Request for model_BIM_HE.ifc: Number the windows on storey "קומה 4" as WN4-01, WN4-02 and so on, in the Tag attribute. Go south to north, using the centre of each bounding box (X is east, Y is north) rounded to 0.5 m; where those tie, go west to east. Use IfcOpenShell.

First a look at what the model holds.

```python
import ifcopenshell
import ifcopenshell.util.element
import ifcopenshell.util.placement

model = ifcopenshell.open("model_BIM_HE.ifc")
print(model.schema)
storey = next(s for s in model.by_type("IfcBuildingStorey") if s.Name == "קומה 4")
windows = [e for e in ifcopenshell.util.element.get_decomposition(storey) if e.is_a("IfcWindow")]
for e in sorted(windows, key=lambda e: e.id()):
    origin = ifcopenshell.util.placement.get_local_placement(e.ObjectPlacement)[:3, 3]
    print(e.id(), e.Tag, e.Name, origin.round(2) + 0.0, sep=" | ")
```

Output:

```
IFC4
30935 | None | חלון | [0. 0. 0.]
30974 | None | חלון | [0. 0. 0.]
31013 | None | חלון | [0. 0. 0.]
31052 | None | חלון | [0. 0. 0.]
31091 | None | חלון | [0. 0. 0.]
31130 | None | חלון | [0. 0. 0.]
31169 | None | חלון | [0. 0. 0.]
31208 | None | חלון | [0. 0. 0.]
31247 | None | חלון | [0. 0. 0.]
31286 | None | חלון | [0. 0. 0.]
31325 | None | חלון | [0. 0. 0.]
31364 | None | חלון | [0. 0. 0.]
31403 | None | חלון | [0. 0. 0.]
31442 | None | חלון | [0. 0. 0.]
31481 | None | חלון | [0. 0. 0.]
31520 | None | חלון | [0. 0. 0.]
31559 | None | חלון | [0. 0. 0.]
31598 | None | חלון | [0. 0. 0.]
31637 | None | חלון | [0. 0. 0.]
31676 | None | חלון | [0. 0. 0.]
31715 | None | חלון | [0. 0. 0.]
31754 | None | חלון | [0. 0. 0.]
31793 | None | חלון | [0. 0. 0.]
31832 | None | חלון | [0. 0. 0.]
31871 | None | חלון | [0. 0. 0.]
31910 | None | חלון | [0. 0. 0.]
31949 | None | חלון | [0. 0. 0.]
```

```python
import ifcopenshell
import ifcopenshell.geom
import ifcopenshell.util.element
import ifcopenshell.util.shape

model = ifcopenshell.open("model_BIM_HE.ifc")
settings = ifcopenshell.geom.settings()
settings.set("use-world-coords", True)


def centre(element):
    shape = ifcopenshell.geom.create_shape(settings, element)
    return ifcopenshell.util.shape.get_bbox_centroid(shape.geometry)


storey = next(s for s in model.by_type("IfcBuildingStorey") if s.Name == "קומה 4")
windows = [e for e in ifcopenshell.util.element.get_decomposition(storey) if e.is_a("IfcWindow")]

# Insertion points can sit at a corner or the storey origin, so sort by the geometry (in metres).
centres = {e: centre(e) for e in windows}
windows.sort(key=lambda e: (round(centres[e][1] / 0.5), centres[e][0]))

for i, e in enumerate(windows, start=1):
    number = f"WN4-{i:02d}"
    e.Tag = number
    print(e.id(), number)

model.write("model_BIM_HE_rev.ifc")
```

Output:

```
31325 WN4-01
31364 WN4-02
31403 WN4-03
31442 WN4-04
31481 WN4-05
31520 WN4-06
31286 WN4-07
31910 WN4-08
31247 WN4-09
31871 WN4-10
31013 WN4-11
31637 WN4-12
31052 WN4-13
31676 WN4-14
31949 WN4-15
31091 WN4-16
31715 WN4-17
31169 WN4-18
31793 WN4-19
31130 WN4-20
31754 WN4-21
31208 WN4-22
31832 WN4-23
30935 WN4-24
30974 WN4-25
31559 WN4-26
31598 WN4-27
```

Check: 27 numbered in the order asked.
